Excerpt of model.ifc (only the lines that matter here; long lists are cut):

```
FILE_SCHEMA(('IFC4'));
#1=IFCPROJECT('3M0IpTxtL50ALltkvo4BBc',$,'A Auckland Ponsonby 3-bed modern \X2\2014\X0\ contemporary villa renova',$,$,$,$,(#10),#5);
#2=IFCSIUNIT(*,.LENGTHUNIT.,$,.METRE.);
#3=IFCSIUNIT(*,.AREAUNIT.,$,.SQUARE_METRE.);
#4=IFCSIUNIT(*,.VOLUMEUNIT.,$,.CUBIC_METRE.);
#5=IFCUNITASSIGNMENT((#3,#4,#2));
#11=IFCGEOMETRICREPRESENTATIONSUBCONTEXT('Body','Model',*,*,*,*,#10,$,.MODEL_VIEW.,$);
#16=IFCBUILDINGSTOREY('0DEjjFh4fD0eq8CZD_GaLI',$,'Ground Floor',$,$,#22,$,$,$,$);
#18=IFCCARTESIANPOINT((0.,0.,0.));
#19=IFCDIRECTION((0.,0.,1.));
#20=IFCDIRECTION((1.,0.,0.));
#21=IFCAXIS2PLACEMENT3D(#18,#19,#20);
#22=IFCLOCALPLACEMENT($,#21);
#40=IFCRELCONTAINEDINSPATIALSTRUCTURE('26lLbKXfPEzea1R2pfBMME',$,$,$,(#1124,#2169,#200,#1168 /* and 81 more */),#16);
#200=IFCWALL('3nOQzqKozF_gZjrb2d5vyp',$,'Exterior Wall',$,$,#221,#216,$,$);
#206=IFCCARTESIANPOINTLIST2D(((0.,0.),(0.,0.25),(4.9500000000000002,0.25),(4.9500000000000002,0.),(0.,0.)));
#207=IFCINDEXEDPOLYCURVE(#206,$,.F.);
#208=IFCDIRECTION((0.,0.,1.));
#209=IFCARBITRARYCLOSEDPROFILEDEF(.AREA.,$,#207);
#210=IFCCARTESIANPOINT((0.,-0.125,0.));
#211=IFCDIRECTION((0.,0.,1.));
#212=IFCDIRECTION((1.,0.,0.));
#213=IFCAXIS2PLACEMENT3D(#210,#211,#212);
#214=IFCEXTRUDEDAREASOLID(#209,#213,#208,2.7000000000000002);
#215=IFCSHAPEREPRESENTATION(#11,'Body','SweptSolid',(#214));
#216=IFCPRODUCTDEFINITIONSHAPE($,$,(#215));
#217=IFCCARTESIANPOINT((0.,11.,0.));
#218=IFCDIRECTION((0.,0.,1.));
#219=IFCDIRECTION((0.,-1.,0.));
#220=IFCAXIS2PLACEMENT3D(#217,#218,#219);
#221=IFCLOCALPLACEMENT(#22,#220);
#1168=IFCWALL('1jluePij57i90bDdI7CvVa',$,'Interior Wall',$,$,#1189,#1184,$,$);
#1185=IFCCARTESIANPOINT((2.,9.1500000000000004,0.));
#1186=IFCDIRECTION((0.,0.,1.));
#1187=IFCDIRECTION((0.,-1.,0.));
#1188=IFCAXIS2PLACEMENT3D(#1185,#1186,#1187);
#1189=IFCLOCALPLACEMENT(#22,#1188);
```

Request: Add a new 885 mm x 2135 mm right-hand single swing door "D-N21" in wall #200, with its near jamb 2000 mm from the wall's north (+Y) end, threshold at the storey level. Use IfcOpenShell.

```python
import numpy as np
import ifcopenshell
import ifcopenshell.api.feature
import ifcopenshell.api.geometry
import ifcopenshell.api.root
import ifcopenshell.api.spatial
import ifcopenshell.geom
import ifcopenshell.util.element
import ifcopenshell.util.placement
import ifcopenshell.util.representation
import ifcopenshell.util.shape
import ifcopenshell.util.unit

model = ifcopenshell.open("model.ifc")
unit_scale = ifcopenshell.util.unit.calculate_unit_scale(model)
settings = ifcopenshell.geom.settings()


def volume(element):
    """Net volume in cubic metres, openings subtracted."""
    shape = ifcopenshell.geom.create_shape(settings, element)
    return ifcopenshell.util.shape.get_volume(shape.geometry)


wall = model.by_id(200)
storey = ifcopenshell.util.element.get_container(wall, ifc_class="IfcBuildingStorey")
context = ifcopenshell.util.representation.get_context(model, "Model", "Body", "MODEL_VIEW")
before = volume(wall)

width, height, from_end, sill = 0.885, 2.135, 2, 0.0  # metres

# The wall runs along its own X axis, and the end named is its -X end.
wall_shape = ifcopenshell.geom.create_shape(settings, wall)
x, y, z = ifcopenshell.util.shape.get_vertices(wall_shape.geometry).T
start = x.min() + from_end
face, thickness = float(y.min()), float(y.max() - y.min())
wall_matrix = ifcopenshell.util.placement.get_local_placement(wall.ObjectPlacement)
level = ifcopenshell.util.placement.get_local_placement(storey.ObjectPlacement)[2, 3]


def in_wall(x, y):
    """Placement at x, y metres in the wall's axes, at sill height."""
    matrix = wall_matrix.copy()
    matrix[:, 3] = wall_matrix @ np.array([x / unit_scale, y / unit_scale, 0.0, 1.0])
    matrix[2, 3] = level + sill / unit_scale
    return matrix


# Opening: a box that overshoots both wall faces by 50 mm.
opening = ifcopenshell.api.root.create_entity(model, ifc_class="IfcOpeningElement", predefined_type="OPENING")
box = ifcopenshell.api.geometry.add_wall_representation(
    model, context=context, length=width, height=height, thickness=thickness + 0.1
)
ifcopenshell.api.geometry.assign_representation(model, product=opening, representation=box)
ifcopenshell.api.geometry.edit_object_placement(model, product=opening, matrix=in_wall(start, face - 0.05), is_si=False)
ifcopenshell.api.feature.add_feature(model, feature=opening, element=wall)

door = ifcopenshell.api.root.create_entity(model, ifc_class="IfcDoor", name="D-N21", predefined_type="DOOR")
door.OverallWidth, door.OverallHeight = width / unit_scale, height / unit_scale
door.OperationType = "SINGLE_SWING_RIGHT"
body = ifcopenshell.api.geometry.add_door_representation(
    model,
    context=context,
    overall_width=door.OverallWidth,
    overall_height=door.OverallHeight,
    operation_type="SINGLE_SWING_RIGHT",
    lining_properties={"LiningDepth": thickness / unit_scale, "ThresholdDepth": thickness / unit_scale},
)
ifcopenshell.api.geometry.assign_representation(model, product=door, representation=body)
ifcopenshell.api.spatial.assign_container(model, products=[door], relating_structure=storey)
ifcopenshell.api.feature.add_filling(model, opening=opening, element=door)

# The lining spans the wall, so the door starts at the wall face.
ifcopenshell.api.geometry.edit_object_placement(model, product=door, matrix=in_wall(start, face), is_si=False)

after = volume(wall)

print(f"wall volume {before:.3f} -> {after:.3f} m3")

model.write("model-out.ifc")
```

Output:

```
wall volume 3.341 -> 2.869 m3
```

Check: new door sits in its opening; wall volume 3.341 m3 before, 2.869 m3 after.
